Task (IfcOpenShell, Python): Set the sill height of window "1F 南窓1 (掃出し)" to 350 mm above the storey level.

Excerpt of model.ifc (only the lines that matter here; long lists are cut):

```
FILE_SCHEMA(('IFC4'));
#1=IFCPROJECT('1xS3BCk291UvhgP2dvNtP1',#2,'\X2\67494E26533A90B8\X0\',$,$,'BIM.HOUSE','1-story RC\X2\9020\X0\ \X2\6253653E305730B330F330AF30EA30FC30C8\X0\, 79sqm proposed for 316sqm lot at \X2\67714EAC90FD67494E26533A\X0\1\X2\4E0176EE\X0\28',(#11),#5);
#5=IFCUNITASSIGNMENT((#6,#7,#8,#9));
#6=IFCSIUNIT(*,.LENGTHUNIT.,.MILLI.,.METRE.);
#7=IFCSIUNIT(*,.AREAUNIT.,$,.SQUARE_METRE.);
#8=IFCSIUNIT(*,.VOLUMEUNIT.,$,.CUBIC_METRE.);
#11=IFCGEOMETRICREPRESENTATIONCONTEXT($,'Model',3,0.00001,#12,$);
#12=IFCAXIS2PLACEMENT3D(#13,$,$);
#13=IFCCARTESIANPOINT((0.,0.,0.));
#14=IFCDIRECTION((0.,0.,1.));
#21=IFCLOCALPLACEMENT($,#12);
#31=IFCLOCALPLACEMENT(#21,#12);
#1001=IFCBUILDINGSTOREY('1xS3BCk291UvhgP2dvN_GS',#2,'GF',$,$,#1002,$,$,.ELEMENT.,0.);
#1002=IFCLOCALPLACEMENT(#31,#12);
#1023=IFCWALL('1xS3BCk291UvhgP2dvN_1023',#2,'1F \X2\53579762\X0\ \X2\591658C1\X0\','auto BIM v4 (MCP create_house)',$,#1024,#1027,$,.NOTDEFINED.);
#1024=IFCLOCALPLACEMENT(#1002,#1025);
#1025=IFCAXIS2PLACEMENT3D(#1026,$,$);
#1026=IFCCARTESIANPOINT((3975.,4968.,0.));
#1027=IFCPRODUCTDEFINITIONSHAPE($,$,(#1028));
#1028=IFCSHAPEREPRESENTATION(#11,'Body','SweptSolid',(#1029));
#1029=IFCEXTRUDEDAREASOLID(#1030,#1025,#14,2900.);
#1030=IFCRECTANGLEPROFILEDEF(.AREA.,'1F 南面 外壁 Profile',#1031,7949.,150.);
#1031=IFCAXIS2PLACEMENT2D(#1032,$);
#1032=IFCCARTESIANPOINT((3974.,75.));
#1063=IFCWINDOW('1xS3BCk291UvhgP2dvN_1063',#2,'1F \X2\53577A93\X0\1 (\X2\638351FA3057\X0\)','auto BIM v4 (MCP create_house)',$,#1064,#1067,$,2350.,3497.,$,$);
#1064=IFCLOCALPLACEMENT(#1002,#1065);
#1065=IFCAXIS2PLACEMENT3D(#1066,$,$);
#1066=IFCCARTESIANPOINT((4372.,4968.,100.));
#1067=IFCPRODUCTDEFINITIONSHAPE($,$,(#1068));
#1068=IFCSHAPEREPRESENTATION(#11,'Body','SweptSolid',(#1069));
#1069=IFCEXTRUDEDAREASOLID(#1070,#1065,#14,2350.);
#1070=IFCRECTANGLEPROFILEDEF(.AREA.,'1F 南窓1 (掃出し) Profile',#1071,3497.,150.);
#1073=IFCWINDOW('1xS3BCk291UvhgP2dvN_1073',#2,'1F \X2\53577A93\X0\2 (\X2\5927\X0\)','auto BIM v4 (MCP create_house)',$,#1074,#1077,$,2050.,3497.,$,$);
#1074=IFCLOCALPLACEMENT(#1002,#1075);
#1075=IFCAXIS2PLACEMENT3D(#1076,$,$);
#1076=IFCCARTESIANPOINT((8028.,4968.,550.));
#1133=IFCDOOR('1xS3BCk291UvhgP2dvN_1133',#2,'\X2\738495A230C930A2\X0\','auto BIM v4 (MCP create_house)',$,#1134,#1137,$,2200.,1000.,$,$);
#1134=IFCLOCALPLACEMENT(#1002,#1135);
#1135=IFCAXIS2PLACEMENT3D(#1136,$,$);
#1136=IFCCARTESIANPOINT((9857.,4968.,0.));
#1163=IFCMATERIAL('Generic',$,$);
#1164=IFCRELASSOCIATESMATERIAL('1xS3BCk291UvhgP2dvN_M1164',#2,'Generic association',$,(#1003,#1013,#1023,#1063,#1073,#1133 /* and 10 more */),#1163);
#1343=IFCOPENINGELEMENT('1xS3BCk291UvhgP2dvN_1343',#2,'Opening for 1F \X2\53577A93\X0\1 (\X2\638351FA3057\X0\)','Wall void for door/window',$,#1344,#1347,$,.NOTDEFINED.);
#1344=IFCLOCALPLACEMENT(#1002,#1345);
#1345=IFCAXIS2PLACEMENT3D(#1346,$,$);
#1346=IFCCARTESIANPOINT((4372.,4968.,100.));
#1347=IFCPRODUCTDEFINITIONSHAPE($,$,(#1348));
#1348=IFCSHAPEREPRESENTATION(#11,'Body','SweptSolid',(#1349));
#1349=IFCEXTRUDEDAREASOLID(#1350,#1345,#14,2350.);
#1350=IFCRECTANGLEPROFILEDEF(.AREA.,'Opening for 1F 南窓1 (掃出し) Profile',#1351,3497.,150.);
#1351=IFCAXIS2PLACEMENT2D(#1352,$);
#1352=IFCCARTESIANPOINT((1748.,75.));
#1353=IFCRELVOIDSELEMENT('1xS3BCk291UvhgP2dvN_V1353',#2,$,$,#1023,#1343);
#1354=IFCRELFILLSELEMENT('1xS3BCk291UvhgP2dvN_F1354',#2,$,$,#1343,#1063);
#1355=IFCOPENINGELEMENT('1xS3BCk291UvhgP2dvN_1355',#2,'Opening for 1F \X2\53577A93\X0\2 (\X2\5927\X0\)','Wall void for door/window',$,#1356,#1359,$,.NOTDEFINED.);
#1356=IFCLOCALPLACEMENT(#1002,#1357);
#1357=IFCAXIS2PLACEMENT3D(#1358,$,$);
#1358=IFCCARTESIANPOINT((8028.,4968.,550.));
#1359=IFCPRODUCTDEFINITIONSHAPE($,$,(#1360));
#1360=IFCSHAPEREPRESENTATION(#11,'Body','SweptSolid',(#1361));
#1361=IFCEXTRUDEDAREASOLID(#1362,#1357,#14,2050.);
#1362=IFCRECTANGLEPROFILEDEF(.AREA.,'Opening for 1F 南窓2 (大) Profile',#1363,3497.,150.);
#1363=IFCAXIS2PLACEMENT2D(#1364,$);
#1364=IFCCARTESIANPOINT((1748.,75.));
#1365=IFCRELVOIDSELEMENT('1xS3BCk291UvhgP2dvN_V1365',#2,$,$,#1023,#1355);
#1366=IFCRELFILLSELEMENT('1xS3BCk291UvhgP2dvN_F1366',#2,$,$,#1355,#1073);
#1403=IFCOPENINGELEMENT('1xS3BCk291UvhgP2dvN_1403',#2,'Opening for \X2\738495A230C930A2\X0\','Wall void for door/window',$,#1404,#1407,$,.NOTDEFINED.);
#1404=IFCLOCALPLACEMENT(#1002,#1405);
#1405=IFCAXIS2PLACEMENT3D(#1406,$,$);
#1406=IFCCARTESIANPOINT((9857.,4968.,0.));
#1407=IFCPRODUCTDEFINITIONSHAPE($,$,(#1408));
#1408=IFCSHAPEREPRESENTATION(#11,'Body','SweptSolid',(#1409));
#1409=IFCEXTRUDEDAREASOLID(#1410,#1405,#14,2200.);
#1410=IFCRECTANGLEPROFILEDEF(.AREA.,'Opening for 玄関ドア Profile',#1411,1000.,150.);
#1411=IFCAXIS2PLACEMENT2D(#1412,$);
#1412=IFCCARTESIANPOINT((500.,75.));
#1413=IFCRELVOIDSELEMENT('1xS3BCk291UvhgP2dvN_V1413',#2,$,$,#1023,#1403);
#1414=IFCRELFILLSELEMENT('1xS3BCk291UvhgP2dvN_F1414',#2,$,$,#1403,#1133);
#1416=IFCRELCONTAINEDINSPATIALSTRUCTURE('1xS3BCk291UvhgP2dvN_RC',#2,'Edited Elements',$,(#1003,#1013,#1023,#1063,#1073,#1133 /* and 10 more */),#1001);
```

```python
import numpy as np
import ifcopenshell
import ifcopenshell.api.geometry
import ifcopenshell.geom
import ifcopenshell.util.element
import ifcopenshell.util.placement
import ifcopenshell.util.shape
import ifcopenshell.util.unit

model = ifcopenshell.open("model.ifc")
unit_scale = ifcopenshell.util.unit.calculate_unit_scale(model)

window = model.by_guid("1xS3BCk291UvhgP2dvN_1063")
opening = window.FillsVoids[0].RelatingOpeningElement
storey = ifcopenshell.util.element.get_container(window, ifc_class="IfcBuildingStorey")
level = ifcopenshell.util.placement.get_local_placement(storey.ObjectPlacement)[2, 3]

# The opening's origin need not be at the sill, so measure its lowest point.
shape = ifcopenshell.geom.create_shape(ifcopenshell.geom.settings(), opening)
bottom = ifcopenshell.util.shape.get_shape_bottom_elevation(shape, shape.geometry) / unit_scale
dz = level + 0.35 / unit_scale - bottom

shift = np.array([0.0, 0.0, dz])
# The window is not placed relative to its opening, so move both.
for product in (opening, window):
    matrix = ifcopenshell.util.placement.get_local_placement(product.ObjectPlacement)
    matrix[:3, 3] += shift
    ifcopenshell.api.geometry.edit_object_placement(model, product=product, matrix=matrix, is_si=False)

print(f"moved by {dz * unit_scale:+.3f} m")

model.write("model-out.ifc")
```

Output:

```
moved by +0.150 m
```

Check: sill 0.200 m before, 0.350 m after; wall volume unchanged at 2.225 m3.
